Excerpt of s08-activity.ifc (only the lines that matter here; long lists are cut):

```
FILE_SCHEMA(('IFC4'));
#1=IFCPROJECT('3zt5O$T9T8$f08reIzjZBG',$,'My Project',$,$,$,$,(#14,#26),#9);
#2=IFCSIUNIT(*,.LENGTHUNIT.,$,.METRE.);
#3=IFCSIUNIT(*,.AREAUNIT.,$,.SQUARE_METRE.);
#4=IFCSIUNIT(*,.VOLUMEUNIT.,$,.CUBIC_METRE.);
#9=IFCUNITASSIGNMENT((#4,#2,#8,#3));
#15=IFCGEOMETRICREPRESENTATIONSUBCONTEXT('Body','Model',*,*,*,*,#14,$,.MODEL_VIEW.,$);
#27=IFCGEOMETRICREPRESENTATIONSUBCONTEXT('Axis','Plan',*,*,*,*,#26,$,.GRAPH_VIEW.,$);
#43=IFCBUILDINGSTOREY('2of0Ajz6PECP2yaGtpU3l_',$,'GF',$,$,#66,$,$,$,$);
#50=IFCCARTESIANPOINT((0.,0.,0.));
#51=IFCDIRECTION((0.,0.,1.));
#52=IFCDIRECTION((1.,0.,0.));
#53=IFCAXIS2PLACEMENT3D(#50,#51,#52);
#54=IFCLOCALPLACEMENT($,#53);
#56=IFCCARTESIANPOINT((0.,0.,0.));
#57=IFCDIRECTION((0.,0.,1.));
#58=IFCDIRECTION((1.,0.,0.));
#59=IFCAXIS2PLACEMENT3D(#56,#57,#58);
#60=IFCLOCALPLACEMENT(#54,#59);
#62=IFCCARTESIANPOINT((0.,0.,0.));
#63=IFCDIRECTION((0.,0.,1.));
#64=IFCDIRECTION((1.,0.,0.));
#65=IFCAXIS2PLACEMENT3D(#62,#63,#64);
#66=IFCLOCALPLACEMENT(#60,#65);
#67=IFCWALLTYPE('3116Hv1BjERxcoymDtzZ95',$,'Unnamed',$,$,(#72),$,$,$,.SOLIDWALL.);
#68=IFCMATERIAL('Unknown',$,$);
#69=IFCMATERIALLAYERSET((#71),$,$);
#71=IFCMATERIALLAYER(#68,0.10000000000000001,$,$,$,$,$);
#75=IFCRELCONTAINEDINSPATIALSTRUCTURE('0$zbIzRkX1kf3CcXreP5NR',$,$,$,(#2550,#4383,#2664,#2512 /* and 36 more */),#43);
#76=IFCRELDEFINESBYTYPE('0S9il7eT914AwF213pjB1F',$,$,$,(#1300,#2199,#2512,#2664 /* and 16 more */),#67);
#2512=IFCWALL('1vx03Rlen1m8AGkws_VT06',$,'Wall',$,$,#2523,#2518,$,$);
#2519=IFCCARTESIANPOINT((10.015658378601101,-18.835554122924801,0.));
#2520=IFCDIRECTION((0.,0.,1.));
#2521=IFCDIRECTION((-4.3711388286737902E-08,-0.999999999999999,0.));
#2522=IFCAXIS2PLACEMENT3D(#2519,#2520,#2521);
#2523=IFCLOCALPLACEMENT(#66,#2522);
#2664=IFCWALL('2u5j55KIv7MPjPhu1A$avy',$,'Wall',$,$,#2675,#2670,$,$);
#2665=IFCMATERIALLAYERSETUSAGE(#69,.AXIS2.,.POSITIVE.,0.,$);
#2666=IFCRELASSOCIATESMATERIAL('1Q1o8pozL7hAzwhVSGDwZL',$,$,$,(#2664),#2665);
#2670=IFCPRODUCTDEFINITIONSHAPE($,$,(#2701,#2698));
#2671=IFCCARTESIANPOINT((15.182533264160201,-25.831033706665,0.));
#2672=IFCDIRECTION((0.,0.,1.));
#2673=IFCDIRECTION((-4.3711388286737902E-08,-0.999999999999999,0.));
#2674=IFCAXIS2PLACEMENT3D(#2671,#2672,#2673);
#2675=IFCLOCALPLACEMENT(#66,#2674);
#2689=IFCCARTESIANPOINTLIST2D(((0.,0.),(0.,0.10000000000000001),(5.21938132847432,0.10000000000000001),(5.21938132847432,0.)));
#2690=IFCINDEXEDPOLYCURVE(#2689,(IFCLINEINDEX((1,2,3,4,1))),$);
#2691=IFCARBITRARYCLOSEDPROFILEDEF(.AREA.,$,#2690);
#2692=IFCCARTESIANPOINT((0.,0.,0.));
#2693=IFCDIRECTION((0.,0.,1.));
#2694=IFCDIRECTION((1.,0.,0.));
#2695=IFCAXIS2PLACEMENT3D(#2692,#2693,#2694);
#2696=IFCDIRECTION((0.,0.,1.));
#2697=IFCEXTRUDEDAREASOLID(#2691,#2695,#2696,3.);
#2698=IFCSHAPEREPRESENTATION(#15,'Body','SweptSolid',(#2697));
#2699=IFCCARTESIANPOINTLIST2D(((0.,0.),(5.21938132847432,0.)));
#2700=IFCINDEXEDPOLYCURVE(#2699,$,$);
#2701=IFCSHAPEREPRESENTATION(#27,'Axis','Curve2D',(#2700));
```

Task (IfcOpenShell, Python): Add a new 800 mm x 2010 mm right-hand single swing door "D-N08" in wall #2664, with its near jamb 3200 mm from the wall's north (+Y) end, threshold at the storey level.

```python
import numpy as np
import ifcopenshell
import ifcopenshell.api.feature
import ifcopenshell.api.geometry
import ifcopenshell.api.root
import ifcopenshell.api.spatial
import ifcopenshell.geom
import ifcopenshell.util.element
import ifcopenshell.util.placement
import ifcopenshell.util.representation
import ifcopenshell.util.shape
import ifcopenshell.util.unit

model = ifcopenshell.open("s08-activity.ifc")
unit_scale = ifcopenshell.util.unit.calculate_unit_scale(model)
settings = ifcopenshell.geom.settings()


def volume(element):
    """Net volume in cubic metres, openings subtracted."""
    shape = ifcopenshell.geom.create_shape(settings, element)
    return ifcopenshell.util.shape.get_volume(shape.geometry)


wall = model.by_guid("2u5j55KIv7MPjPhu1A$avy")
storey = ifcopenshell.util.element.get_container(wall, ifc_class="IfcBuildingStorey")
context = ifcopenshell.util.representation.get_context(model, "Model", "Body", "MODEL_VIEW")
before = volume(wall)

width, height, from_end, sill = 0.8, 2.01, 3.2, 0.0  # metres

# The wall runs along its own X axis, and the end named is its -X end.
wall_shape = ifcopenshell.geom.create_shape(settings, wall)
x, y, z = ifcopenshell.util.shape.get_vertices(wall_shape.geometry).T
start = x.min() + from_end
face, thickness = float(y.min()), float(y.max() - y.min())
wall_matrix = ifcopenshell.util.placement.get_local_placement(wall.ObjectPlacement)
level = ifcopenshell.util.placement.get_local_placement(storey.ObjectPlacement)[2, 3]


def in_wall(x, y):
    """Placement at x, y metres in the wall's axes, at sill height."""
    matrix = wall_matrix.copy()
    matrix[:, 3] = wall_matrix @ np.array([x / unit_scale, y / unit_scale, 0.0, 1.0])
    matrix[2, 3] = level + sill / unit_scale
    return matrix


# Opening: a box that overshoots both wall faces by 50 mm.
opening = ifcopenshell.api.root.create_entity(model, ifc_class="IfcOpeningElement", predefined_type="OPENING")
box = ifcopenshell.api.geometry.add_wall_representation(
    model, context=context, length=width, height=height, thickness=thickness + 0.1
)
ifcopenshell.api.geometry.assign_representation(model, product=opening, representation=box)
ifcopenshell.api.geometry.edit_object_placement(model, product=opening, matrix=in_wall(start, face - 0.05), is_si=False)
ifcopenshell.api.feature.add_feature(model, feature=opening, element=wall)

door = ifcopenshell.api.root.create_entity(model, ifc_class="IfcDoor", name="D-N08", predefined_type="DOOR")
door.OverallWidth, door.OverallHeight = width / unit_scale, height / unit_scale
door.OperationType = "SINGLE_SWING_RIGHT"
body = ifcopenshell.api.geometry.add_door_representation(
    model,
    context=context,
    overall_width=door.OverallWidth,
    overall_height=door.OverallHeight,
    operation_type="SINGLE_SWING_RIGHT",
    lining_properties={"LiningDepth": thickness / unit_scale, "ThresholdDepth": thickness / unit_scale},
)
ifcopenshell.api.geometry.assign_representation(model, product=door, representation=body)
ifcopenshell.api.spatial.assign_container(model, products=[door], relating_structure=storey)
ifcopenshell.api.feature.add_filling(model, opening=opening, element=door)

# The lining spans the wall, so the door starts at the wall face.
ifcopenshell.api.geometry.edit_object_placement(model, product=door, matrix=in_wall(start, face), is_si=False)

after = volume(wall)

print(f"wall volume {before:.3f} -> {after:.3f} m3")

model.write("s08-activity_rev.ifc")
```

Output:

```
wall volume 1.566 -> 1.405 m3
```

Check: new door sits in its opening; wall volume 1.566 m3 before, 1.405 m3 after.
